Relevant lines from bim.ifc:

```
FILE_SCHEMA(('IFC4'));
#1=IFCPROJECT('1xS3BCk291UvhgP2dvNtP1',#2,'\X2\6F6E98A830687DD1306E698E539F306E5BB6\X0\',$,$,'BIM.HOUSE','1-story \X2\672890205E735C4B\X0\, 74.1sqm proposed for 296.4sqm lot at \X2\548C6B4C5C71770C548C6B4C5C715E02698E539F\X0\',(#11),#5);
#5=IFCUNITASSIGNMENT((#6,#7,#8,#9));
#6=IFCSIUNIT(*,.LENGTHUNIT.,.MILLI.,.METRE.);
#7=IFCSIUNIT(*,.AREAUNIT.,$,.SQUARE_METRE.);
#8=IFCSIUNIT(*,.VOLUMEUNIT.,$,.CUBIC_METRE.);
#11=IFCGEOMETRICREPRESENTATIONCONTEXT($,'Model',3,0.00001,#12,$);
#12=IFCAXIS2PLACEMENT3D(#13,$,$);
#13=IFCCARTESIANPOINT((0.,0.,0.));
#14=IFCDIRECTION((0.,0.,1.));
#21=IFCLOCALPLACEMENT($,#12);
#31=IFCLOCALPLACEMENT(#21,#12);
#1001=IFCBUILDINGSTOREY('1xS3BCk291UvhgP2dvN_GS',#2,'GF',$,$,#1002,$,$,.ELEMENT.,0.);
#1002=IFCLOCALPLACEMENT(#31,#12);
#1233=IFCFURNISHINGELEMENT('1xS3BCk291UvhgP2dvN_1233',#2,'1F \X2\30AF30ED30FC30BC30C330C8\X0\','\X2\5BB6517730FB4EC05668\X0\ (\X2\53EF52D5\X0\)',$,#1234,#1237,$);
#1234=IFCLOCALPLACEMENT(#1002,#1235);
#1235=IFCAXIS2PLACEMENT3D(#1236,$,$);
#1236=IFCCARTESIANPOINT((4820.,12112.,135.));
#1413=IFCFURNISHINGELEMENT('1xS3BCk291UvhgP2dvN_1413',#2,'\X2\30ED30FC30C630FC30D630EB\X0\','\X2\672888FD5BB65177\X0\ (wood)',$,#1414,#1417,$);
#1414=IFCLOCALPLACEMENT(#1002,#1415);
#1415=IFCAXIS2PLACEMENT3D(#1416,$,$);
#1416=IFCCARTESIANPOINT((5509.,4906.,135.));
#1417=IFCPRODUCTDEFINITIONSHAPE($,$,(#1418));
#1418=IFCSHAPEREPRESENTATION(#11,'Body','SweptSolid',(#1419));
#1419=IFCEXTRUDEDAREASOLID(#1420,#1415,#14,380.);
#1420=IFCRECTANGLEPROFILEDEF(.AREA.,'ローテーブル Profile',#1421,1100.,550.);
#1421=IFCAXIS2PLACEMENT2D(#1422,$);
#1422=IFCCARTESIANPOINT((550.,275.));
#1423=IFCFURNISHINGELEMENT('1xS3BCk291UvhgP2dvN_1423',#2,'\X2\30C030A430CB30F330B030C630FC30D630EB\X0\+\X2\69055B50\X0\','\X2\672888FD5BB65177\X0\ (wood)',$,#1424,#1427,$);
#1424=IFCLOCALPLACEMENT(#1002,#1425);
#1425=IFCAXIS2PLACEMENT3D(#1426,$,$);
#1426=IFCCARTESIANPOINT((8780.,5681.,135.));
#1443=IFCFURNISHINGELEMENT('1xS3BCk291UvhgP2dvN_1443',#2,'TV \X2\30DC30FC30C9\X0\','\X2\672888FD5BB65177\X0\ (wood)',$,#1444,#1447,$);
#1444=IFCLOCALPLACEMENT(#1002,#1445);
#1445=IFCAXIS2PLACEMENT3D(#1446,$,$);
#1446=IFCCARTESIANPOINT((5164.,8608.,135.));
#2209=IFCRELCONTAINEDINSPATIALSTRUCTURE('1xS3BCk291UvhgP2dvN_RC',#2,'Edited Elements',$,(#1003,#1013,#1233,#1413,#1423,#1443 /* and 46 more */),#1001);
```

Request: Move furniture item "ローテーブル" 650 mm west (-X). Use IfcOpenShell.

```python
import ifcopenshell
import ifcopenshell.api.geometry
import ifcopenshell.util.placement
import ifcopenshell.util.unit

model = ifcopenshell.open("bim.ifc")
unit_scale = ifcopenshell.util.unit.calculate_unit_scale(model)

item = model.by_id(1413)
matrix = ifcopenshell.util.placement.get_local_placement(item.ObjectPlacement)
matrix[0, 3] -= 0.65 / unit_scale
ifcopenshell.api.geometry.edit_object_placement(model, product=item, matrix=matrix, is_si=False)

print(ifcopenshell.util.placement.get_local_placement(item.ObjectPlacement).round(3) + 0.0)

model.write("bim_updated.ifc")
```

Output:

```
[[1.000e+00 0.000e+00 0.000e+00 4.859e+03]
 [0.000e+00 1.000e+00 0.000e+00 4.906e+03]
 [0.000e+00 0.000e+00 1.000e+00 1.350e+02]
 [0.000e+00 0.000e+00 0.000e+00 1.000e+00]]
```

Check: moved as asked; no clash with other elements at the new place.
